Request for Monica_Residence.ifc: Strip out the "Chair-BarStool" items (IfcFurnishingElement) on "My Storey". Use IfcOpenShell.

First a look at what the model holds.

```python
import ifcopenshell
import ifcopenshell.util.element

model = ifcopenshell.open("Monica_Residence.ifc")
print(model.schema)
storey = next(s for s in model.by_type("IfcBuildingStorey") if s.Name == "My Storey")
furniture = [e for e in ifcopenshell.util.element.get_decomposition(storey) if e.is_a("IfcFurnishingElement")]
seen = {}
for e in furniture:
    element_type = ifcopenshell.util.element.get_type(e)
    name = element_type.Name if element_type not in (None, e) else None
    seen[name] = seen.get(name, 0) + 1
for name, count in sorted(seen.items(), key=str):
    print(count, "x", name)
```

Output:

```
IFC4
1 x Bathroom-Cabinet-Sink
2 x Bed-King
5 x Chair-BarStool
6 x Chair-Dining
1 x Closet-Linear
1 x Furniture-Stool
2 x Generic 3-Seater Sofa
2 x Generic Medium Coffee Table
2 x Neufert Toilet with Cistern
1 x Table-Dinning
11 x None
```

```python
import ifcopenshell
import ifcopenshell.api.root
import ifcopenshell.util.element

model = ifcopenshell.open("Monica_Residence.ifc")

storey = next(s for s in model.by_type("IfcBuildingStorey") if s.Name == "My Storey")
furniture = [e for e in ifcopenshell.util.element.get_decomposition(storey) if e.is_a("IfcFurnishingElement")]
targets = [e for e in furniture if (t := ifcopenshell.util.element.get_type(e)) not in (None, e) and t.Name == "Chair-BarStool"]

for e in targets:
    ifcopenshell.api.root.remove_product(model, product=e)
print(len(targets), "removed")

model.write("Monica_Residence_rev.ifc")
```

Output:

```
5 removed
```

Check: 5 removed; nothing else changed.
